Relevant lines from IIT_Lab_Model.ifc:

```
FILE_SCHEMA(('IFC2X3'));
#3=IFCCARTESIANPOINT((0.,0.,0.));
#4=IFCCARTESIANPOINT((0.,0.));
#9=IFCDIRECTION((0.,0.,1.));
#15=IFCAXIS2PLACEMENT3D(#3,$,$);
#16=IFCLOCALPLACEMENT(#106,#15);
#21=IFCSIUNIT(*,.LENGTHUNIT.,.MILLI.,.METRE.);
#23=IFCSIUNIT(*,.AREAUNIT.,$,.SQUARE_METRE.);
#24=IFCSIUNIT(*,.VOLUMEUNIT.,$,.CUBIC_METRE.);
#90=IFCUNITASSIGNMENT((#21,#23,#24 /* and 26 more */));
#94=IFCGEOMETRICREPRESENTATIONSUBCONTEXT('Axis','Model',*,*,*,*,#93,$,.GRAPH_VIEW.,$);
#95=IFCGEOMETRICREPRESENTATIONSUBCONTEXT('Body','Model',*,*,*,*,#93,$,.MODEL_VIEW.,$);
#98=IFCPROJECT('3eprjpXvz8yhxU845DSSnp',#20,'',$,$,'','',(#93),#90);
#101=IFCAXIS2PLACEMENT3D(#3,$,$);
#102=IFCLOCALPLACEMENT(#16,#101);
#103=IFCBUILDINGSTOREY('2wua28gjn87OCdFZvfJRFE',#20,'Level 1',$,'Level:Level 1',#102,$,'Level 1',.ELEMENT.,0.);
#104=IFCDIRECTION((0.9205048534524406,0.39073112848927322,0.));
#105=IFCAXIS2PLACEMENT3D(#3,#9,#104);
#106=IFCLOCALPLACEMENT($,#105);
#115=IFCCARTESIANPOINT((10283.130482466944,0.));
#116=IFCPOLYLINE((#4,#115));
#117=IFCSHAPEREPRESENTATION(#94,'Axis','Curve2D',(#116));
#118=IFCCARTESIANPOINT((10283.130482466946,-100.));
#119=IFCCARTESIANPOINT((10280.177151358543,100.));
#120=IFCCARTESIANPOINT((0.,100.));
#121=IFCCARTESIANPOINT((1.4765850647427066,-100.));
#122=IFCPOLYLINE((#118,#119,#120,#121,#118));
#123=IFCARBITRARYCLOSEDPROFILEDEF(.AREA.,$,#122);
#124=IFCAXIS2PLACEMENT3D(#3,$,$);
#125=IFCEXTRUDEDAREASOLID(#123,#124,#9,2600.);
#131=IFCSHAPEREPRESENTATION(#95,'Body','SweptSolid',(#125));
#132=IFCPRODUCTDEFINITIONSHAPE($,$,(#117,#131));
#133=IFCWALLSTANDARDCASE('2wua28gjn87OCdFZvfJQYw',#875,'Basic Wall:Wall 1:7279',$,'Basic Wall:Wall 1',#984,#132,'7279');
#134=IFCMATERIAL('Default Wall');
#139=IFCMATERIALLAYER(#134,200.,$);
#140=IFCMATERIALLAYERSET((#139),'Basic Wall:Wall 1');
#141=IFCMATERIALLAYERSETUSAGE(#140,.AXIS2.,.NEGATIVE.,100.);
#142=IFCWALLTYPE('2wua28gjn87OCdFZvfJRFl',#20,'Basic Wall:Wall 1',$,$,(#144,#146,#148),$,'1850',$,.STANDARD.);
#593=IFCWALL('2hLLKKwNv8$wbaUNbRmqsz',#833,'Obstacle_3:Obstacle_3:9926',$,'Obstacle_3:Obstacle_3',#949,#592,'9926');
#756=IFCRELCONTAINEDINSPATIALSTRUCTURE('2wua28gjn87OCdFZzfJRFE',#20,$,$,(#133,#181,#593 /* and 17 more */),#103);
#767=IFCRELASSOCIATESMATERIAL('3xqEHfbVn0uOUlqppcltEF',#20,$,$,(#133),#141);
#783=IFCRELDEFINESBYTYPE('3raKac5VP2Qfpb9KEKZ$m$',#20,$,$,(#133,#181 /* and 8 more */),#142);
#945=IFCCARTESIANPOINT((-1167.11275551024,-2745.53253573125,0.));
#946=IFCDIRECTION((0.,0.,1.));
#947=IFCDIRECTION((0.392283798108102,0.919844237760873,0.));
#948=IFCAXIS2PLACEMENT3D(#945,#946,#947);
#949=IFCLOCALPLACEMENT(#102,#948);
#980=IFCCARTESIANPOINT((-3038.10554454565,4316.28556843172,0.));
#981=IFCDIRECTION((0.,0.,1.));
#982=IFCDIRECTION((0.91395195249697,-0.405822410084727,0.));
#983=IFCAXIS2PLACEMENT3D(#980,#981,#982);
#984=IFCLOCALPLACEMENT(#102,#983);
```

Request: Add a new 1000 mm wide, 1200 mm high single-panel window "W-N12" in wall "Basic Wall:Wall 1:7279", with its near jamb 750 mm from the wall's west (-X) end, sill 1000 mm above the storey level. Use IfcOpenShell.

```python
import numpy as np
import ifcopenshell
import ifcopenshell.api.feature
import ifcopenshell.api.geometry
import ifcopenshell.api.root
import ifcopenshell.api.spatial
import ifcopenshell.api.type
import ifcopenshell.geom
import ifcopenshell.util.element
import ifcopenshell.util.placement
import ifcopenshell.util.representation
import ifcopenshell.util.shape
import ifcopenshell.util.unit

model = ifcopenshell.open("IIT_Lab_Model.ifc")
unit_scale = ifcopenshell.util.unit.calculate_unit_scale(model)
settings = ifcopenshell.geom.settings()


def volume(element):
    """Net volume in cubic metres, openings subtracted."""
    shape = ifcopenshell.geom.create_shape(settings, element)
    return ifcopenshell.util.shape.get_volume(shape.geometry)


wall = model.by_guid("2wua28gjn87OCdFZvfJQYw")
storey = ifcopenshell.util.element.get_container(wall, ifc_class="IfcBuildingStorey")
context = ifcopenshell.util.representation.get_context(model, "Model", "Body", "MODEL_VIEW")
before = volume(wall)

width, height, from_end, sill = 1, 1.2, 0.75, 1  # metres

# The wall runs along its own X axis, and the end named is its -X end.
wall_shape = ifcopenshell.geom.create_shape(settings, wall)
x, y, z = ifcopenshell.util.shape.get_vertices(wall_shape.geometry).T
start = x.min() + from_end
face, thickness = float(y.min()), float(y.max() - y.min())
wall_matrix = ifcopenshell.util.placement.get_local_placement(wall.ObjectPlacement)
level = ifcopenshell.util.placement.get_local_placement(storey.ObjectPlacement)[2, 3]


def in_wall(x, y):
    """Placement at x, y metres in the wall's axes, at sill height."""
    matrix = wall_matrix.copy()
    matrix[:, 3] = wall_matrix @ np.array([x / unit_scale, y / unit_scale, 0.0, 1.0])
    matrix[2, 3] = level + sill / unit_scale
    return matrix


# Opening: a box that overshoots both wall faces by 50 mm.
opening = ifcopenshell.api.root.create_entity(model, ifc_class="IfcOpeningElement")
box = ifcopenshell.api.geometry.add_wall_representation(
    model, context=context, length=width, height=height, thickness=thickness + 0.1
)
ifcopenshell.api.geometry.assign_representation(model, product=opening, representation=box)
ifcopenshell.api.geometry.edit_object_placement(model, product=opening, matrix=in_wall(start, face - 0.05), is_si=False)
ifcopenshell.api.feature.add_feature(model, feature=opening, element=wall)

window = ifcopenshell.api.root.create_entity(model, ifc_class="IfcWindow", name="W-N12")
window.OverallWidth, window.OverallHeight = width / unit_scale, height / unit_scale
body = ifcopenshell.api.geometry.add_window_representation(
    model,
    context=context,
    overall_width=window.OverallWidth,
    overall_height=window.OverallHeight,
    partition_type="SINGLE_PANEL",
)
ifcopenshell.api.geometry.assign_representation(model, product=window, representation=body)
ifcopenshell.api.spatial.assign_container(model, products=[window], relating_structure=storey)
fills = ifcopenshell.api.feature.add_filling(model, opening=opening, element=window)
fills.OwnerHistory = window.OwnerHistory  # required in IFC2X3

# IFC2X3 keeps the operation on the window style.
style = ifcopenshell.api.root.create_entity(model, ifc_class="IfcWindowStyle", name="W-N12")
style.OperationType, style.ConstructionType = "SINGLE_PANEL", "NOTDEFINED"
style.ParameterTakesPrecedence = style.Sizeable = False
ifcopenshell.api.type.assign_type(model, related_objects=[window], relating_type=style)

# Centre the window in the wall's thickness.
ifcopenshell.api.geometry.edit_object_placement(model, product=window, matrix=in_wall(start, face), is_si=False)
window_shape = ifcopenshell.geom.create_shape(settings, window)
depth = ifcopenshell.util.shape.get_vertices(window_shape.geometry)[:, 1]
offset = face + thickness / 2 - (depth.min() + depth.max()) / 2
ifcopenshell.api.geometry.edit_object_placement(model, product=window, matrix=in_wall(start, offset), is_si=False)

after = volume(wall)

print(f"wall volume {before:.3f} -> {after:.3f} m3")

model.write("IIT_Lab_Model_edited.ifc")
```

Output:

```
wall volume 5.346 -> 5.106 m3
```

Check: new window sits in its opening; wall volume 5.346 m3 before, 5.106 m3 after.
